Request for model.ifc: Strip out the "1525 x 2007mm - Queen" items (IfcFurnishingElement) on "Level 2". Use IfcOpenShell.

First a look at what the model holds.

```python
import ifcopenshell
import ifcopenshell.util.element

model = ifcopenshell.open("model.ifc")
print(model.schema)
storey = next(s for s in model.by_type("IfcBuildingStorey") if s.Name == "Level 2")
furniture = [e for e in ifcopenshell.util.element.get_decomposition(storey) if e.is_a("IfcFurnishingElement")]
seen = {}
for e in furniture:
    element_type = ifcopenshell.util.element.get_type(e)
    name = element_type.Name if element_type not in (None, e) else None
    seen[name] = seen.get(name, 0) + 1
for name, count in sorted(seen.items(), key=str):
    print(count, "x", name)
```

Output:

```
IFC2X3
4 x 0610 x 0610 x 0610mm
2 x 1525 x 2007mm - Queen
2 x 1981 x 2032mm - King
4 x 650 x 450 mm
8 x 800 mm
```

```python
import ifcopenshell
import ifcopenshell.api.root
import ifcopenshell.util.element

model = ifcopenshell.open("model.ifc")

storey = next(s for s in model.by_type("IfcBuildingStorey") if s.Name == "Level 2")
furniture = [e for e in ifcopenshell.util.element.get_decomposition(storey) if e.is_a("IfcFurnishingElement")]
targets = [e for e in furniture if (t := ifcopenshell.util.element.get_type(e)) not in (None, e) and t.Name == "1525 x 2007mm - Queen"]

for e in targets:
    ifcopenshell.api.root.remove_product(model, product=e)
print(len(targets), "removed")

model.write("model-out.ifc")
```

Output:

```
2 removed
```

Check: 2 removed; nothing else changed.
